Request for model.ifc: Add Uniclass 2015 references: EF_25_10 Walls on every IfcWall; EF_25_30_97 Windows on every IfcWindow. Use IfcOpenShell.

First a look at what the model holds.

```python
import ifcopenshell

model = ifcopenshell.open("model.ifc")
print(model.schema)
print("classifications:", [c.Name for c in model.by_type("IfcClassification")])
for ifc_class in ("IfcDoor", "IfcRoof", "IfcStair", "IfcWall", "IfcWindow"):
    print(ifc_class, len(model.by_type(ifc_class)))
```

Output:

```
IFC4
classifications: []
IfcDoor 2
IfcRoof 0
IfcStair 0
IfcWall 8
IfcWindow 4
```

```python
import ifcopenshell
import ifcopenshell.api.classification

model = ifcopenshell.open("model.ifc")

system = ifcopenshell.api.classification.add_classification(model, classification="Uniclass 2015")

codes = {
    "IfcWall": ("EF_25_10", "Walls"),
    "IfcWindow": ("EF_25_30_97", "Windows"),
}
for ifc_class, (code, name) in codes.items():
    products = model.by_type(ifc_class)
    ifcopenshell.api.classification.add_reference(
        model, products=products, classification=system, identification=code, name=name
    )
    print(code, len(products))

model.write("model_edited.ifc")
```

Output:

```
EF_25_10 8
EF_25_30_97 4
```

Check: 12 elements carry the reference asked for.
